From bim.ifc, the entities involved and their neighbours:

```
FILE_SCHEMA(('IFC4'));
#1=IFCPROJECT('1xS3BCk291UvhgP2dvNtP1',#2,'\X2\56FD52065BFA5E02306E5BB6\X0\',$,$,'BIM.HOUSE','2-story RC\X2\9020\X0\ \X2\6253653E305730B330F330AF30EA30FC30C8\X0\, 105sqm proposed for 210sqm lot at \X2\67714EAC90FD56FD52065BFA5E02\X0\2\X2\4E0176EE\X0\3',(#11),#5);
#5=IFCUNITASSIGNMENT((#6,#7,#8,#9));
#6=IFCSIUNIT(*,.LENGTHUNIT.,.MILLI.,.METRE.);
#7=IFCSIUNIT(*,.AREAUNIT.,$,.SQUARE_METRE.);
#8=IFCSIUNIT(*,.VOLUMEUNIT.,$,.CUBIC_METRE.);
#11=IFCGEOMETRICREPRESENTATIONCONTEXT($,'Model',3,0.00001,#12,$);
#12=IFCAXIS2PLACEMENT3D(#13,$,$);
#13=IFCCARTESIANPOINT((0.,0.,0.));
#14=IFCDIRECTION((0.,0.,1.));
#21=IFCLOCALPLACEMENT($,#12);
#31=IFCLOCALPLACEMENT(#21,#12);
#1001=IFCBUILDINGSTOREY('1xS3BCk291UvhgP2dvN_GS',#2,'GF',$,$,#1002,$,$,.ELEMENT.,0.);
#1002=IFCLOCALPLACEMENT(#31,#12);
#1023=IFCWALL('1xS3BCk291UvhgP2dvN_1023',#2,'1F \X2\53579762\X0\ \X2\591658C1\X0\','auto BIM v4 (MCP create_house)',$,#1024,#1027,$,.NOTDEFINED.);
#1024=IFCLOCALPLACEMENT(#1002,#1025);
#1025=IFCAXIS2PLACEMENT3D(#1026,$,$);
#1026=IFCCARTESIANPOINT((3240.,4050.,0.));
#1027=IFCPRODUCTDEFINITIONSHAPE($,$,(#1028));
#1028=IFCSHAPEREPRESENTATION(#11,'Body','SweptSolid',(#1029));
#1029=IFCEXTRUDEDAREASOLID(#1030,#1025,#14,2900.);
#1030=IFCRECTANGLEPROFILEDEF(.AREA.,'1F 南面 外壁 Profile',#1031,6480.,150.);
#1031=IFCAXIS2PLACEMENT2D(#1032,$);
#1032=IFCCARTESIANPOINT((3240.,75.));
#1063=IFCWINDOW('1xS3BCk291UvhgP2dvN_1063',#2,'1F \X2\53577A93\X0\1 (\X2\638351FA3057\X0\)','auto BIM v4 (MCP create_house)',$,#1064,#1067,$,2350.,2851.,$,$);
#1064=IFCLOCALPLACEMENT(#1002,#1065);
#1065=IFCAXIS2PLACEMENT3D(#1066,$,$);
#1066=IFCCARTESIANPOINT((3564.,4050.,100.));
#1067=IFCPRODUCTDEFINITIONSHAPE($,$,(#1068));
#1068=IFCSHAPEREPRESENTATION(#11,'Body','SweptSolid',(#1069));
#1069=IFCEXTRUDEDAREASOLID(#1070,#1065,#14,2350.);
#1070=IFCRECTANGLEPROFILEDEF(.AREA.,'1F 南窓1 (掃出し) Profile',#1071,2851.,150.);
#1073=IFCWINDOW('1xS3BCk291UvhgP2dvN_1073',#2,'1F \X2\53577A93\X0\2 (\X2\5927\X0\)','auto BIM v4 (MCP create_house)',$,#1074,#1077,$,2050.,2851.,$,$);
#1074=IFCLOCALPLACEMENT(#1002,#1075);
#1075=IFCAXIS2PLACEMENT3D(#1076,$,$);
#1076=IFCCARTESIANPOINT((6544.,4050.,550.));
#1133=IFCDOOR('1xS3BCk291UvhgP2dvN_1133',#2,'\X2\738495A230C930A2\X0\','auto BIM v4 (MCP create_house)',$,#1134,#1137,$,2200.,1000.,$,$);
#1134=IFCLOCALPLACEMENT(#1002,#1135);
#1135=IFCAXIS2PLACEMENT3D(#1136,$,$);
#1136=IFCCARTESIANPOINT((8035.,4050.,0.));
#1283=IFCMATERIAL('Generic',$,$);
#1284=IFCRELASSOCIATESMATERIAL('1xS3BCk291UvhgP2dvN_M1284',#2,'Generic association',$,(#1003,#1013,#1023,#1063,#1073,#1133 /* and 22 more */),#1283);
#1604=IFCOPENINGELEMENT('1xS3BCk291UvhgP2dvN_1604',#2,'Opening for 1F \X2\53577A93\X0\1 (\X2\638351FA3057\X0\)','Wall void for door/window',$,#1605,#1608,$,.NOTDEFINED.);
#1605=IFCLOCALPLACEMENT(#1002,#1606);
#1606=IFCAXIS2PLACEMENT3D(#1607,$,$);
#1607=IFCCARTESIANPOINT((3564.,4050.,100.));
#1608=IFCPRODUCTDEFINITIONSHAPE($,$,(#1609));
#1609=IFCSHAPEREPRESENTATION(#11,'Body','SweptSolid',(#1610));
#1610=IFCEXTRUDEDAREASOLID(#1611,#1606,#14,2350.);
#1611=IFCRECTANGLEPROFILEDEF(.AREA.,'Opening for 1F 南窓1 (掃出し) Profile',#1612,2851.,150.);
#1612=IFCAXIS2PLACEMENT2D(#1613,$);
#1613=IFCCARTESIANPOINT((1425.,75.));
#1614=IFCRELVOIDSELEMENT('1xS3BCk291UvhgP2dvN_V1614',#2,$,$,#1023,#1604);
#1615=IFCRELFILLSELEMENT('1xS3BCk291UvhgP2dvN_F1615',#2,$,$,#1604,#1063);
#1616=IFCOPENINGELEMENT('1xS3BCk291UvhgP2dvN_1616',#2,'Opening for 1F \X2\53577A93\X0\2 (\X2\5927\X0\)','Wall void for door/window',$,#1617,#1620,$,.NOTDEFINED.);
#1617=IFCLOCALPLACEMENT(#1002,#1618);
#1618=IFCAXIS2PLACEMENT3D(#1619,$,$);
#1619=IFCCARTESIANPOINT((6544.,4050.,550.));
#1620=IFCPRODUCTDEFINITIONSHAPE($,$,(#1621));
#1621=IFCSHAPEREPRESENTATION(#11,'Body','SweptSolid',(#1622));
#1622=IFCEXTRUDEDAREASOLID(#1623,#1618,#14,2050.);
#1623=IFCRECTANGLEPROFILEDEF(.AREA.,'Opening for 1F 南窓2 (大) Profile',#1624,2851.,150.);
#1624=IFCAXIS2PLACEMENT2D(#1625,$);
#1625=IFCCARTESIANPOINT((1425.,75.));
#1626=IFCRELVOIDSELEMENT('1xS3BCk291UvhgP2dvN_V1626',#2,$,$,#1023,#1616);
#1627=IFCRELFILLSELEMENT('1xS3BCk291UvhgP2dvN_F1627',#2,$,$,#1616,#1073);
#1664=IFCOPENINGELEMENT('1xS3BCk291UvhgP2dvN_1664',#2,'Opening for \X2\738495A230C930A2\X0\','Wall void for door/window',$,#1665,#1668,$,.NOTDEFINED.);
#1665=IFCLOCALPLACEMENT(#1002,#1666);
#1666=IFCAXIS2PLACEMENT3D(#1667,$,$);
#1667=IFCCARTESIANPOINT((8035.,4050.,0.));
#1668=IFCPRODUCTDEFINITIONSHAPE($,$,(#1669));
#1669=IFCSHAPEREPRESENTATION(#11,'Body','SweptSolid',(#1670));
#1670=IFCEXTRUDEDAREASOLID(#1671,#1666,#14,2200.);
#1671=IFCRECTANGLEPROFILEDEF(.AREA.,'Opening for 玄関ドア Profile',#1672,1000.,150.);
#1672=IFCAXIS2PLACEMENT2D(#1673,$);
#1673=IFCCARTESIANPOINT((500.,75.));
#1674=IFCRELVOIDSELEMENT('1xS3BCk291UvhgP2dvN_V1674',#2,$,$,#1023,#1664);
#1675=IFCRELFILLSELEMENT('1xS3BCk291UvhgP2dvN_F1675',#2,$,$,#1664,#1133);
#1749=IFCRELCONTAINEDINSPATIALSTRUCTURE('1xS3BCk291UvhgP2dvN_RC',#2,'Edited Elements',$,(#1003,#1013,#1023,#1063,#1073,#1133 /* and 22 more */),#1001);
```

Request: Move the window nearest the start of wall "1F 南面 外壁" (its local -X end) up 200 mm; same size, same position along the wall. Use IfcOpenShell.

```python
import numpy as np
import ifcopenshell
import ifcopenshell.api.geometry
import ifcopenshell.util.placement
import ifcopenshell.util.unit

model = ifcopenshell.open("bim.ifc")
unit_scale = ifcopenshell.util.unit.calculate_unit_scale(model)

window = model.by_guid("1xS3BCk291UvhgP2dvN_1063")
opening = window.FillsVoids[0].RelatingOpeningElement
dz = 0.2 / unit_scale

shift = np.array([0.0, 0.0, dz])
# The window is not placed relative to its opening, so move both.
for product in (opening, window):
    matrix = ifcopenshell.util.placement.get_local_placement(product.ObjectPlacement)
    matrix[:3, 3] += shift
    ifcopenshell.api.geometry.edit_object_placement(model, product=product, matrix=matrix, is_si=False)

print(f"moved by {dz * unit_scale:+.3f} m")

model.write("bim-out.ifc")
```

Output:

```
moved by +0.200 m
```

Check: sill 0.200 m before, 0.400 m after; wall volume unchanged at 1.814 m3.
